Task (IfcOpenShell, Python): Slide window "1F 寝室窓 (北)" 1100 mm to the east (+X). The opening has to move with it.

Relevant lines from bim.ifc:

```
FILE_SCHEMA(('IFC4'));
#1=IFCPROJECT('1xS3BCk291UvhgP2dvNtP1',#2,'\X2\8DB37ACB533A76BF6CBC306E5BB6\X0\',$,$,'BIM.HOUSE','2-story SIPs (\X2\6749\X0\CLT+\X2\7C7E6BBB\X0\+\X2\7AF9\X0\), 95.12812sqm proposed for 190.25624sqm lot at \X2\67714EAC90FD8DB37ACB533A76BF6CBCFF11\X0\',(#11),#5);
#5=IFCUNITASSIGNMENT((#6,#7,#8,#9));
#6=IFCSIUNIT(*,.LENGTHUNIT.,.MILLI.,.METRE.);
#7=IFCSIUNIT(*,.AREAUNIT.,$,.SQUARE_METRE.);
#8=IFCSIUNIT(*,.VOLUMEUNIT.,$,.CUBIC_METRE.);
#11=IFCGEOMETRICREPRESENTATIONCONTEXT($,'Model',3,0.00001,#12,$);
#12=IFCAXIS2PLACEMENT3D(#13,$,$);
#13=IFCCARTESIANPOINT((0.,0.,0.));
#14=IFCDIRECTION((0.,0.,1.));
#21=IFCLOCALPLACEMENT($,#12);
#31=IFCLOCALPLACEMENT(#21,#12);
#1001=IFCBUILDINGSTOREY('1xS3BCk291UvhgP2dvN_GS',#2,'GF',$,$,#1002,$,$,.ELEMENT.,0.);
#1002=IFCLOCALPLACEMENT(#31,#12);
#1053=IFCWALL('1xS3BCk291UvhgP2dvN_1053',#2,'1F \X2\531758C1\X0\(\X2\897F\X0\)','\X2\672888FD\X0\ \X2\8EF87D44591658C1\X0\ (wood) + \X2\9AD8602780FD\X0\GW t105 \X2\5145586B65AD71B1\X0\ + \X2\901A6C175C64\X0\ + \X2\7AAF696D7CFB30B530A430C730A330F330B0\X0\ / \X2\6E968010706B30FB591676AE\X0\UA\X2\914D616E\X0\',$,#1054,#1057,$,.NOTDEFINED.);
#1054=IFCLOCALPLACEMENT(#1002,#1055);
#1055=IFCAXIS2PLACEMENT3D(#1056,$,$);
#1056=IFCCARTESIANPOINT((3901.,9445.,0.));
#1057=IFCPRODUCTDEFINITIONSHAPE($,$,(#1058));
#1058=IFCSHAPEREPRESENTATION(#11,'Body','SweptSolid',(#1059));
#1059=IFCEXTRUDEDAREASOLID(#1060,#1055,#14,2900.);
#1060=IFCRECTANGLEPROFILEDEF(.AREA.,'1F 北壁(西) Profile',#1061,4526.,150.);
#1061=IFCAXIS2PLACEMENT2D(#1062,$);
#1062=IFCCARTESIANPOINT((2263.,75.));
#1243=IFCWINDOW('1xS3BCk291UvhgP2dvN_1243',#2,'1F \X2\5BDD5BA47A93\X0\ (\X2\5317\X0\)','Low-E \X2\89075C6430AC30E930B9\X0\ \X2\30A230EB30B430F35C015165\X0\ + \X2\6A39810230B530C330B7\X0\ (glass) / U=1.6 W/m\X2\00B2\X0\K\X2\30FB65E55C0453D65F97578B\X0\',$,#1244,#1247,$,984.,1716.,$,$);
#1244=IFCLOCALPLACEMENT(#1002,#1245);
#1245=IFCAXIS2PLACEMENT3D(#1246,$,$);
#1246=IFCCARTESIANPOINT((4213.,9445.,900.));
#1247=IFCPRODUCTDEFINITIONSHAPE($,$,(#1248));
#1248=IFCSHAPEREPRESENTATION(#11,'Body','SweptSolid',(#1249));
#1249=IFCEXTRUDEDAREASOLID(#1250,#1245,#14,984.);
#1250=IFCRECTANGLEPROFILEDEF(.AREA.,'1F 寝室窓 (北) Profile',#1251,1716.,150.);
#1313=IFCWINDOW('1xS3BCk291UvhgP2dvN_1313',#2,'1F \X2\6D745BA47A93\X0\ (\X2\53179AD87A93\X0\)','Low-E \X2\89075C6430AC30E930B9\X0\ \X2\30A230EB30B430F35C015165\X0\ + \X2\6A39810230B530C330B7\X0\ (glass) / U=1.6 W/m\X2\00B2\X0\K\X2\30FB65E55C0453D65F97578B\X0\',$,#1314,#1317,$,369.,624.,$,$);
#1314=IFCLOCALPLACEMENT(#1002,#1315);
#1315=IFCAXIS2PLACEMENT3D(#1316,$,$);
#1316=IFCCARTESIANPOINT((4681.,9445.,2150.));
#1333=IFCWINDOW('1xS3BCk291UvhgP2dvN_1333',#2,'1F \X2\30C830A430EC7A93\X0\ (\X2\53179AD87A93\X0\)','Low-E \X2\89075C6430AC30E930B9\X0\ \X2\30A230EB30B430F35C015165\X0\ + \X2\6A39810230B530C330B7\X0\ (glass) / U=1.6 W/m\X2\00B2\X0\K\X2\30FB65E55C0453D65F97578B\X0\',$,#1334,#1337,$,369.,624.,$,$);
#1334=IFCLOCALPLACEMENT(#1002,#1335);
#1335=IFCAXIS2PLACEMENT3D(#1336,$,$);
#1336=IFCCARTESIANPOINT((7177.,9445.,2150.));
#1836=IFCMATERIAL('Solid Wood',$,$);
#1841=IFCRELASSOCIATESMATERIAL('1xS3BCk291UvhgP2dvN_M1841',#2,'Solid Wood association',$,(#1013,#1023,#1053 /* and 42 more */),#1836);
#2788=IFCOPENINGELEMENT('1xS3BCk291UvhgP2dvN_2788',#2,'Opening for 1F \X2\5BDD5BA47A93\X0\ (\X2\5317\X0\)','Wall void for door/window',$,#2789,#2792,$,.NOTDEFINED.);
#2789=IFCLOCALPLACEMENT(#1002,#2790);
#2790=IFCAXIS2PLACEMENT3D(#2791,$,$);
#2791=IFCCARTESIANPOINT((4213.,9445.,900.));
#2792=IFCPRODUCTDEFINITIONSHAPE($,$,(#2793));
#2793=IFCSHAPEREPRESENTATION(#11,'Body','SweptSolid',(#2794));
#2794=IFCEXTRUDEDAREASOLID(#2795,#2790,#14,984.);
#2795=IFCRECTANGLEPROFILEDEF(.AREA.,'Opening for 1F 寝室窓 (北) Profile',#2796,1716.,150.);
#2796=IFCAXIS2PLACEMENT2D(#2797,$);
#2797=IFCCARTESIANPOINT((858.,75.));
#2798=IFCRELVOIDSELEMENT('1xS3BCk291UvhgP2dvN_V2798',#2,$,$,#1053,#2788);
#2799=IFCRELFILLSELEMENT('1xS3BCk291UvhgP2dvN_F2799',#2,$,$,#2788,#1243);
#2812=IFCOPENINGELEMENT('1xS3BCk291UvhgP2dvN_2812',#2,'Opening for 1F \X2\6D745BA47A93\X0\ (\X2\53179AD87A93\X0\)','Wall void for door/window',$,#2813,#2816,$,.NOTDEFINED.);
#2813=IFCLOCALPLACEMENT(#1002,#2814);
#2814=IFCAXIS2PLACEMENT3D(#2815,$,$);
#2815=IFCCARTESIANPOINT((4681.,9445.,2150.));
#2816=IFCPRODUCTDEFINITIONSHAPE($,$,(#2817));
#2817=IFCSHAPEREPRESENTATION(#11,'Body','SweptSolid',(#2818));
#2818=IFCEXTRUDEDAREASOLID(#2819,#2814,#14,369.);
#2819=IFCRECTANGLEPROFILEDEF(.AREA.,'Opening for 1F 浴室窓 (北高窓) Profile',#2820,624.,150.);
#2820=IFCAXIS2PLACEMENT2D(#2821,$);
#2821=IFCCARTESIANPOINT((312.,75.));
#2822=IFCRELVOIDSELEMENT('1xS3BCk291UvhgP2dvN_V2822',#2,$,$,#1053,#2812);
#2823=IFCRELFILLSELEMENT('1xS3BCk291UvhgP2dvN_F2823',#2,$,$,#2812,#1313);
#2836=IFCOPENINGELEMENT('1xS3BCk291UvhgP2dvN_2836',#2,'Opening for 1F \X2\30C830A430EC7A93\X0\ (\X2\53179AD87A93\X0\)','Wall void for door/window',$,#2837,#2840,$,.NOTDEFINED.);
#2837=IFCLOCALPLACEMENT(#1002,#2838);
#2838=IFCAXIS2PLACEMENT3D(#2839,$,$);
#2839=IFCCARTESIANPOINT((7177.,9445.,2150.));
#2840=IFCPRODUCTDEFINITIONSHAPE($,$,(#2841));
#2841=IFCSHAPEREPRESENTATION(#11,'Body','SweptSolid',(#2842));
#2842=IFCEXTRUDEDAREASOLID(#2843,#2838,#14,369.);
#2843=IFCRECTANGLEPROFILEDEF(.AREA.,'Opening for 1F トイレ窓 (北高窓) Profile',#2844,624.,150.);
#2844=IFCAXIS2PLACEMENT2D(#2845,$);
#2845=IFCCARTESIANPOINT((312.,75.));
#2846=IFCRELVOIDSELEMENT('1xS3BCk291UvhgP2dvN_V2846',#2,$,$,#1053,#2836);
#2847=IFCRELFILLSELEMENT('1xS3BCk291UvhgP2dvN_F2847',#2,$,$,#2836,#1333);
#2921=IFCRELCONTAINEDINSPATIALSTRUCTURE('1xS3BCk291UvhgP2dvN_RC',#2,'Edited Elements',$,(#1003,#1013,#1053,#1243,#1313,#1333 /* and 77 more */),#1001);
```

```python
import ifcopenshell
import ifcopenshell.api.geometry
import ifcopenshell.util.placement
import ifcopenshell.util.unit

model = ifcopenshell.open("bim.ifc")
unit_scale = ifcopenshell.util.unit.calculate_unit_scale(model)

window = model.by_guid("1xS3BCk291UvhgP2dvN_1243")
opening = window.FillsVoids[0].RelatingOpeningElement
wall = opening.VoidsElements[0].RelatingBuildingElement

wall_matrix = ifcopenshell.util.placement.get_local_placement(wall.ObjectPlacement)
shift = wall_matrix[:3, 0] * 1.1 / unit_scale
before = ifcopenshell.util.placement.get_local_placement(window.ObjectPlacement)[:3, 3].copy()

# The window is not placed relative to its opening, so move both.
for product in (opening, window):
    matrix = ifcopenshell.util.placement.get_local_placement(product.ObjectPlacement)
    matrix[:3, 3] += shift
    ifcopenshell.api.geometry.edit_object_placement(model, product=product, matrix=matrix, is_si=False)

after = ifcopenshell.util.placement.get_local_placement(window.ObjectPlacement)[:3, 3]
print("window moved by", (after - before).round(3) + 0.0)

model.write("bim_rev.ifc")
```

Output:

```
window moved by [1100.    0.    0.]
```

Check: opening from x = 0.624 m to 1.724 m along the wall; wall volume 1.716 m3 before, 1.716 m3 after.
